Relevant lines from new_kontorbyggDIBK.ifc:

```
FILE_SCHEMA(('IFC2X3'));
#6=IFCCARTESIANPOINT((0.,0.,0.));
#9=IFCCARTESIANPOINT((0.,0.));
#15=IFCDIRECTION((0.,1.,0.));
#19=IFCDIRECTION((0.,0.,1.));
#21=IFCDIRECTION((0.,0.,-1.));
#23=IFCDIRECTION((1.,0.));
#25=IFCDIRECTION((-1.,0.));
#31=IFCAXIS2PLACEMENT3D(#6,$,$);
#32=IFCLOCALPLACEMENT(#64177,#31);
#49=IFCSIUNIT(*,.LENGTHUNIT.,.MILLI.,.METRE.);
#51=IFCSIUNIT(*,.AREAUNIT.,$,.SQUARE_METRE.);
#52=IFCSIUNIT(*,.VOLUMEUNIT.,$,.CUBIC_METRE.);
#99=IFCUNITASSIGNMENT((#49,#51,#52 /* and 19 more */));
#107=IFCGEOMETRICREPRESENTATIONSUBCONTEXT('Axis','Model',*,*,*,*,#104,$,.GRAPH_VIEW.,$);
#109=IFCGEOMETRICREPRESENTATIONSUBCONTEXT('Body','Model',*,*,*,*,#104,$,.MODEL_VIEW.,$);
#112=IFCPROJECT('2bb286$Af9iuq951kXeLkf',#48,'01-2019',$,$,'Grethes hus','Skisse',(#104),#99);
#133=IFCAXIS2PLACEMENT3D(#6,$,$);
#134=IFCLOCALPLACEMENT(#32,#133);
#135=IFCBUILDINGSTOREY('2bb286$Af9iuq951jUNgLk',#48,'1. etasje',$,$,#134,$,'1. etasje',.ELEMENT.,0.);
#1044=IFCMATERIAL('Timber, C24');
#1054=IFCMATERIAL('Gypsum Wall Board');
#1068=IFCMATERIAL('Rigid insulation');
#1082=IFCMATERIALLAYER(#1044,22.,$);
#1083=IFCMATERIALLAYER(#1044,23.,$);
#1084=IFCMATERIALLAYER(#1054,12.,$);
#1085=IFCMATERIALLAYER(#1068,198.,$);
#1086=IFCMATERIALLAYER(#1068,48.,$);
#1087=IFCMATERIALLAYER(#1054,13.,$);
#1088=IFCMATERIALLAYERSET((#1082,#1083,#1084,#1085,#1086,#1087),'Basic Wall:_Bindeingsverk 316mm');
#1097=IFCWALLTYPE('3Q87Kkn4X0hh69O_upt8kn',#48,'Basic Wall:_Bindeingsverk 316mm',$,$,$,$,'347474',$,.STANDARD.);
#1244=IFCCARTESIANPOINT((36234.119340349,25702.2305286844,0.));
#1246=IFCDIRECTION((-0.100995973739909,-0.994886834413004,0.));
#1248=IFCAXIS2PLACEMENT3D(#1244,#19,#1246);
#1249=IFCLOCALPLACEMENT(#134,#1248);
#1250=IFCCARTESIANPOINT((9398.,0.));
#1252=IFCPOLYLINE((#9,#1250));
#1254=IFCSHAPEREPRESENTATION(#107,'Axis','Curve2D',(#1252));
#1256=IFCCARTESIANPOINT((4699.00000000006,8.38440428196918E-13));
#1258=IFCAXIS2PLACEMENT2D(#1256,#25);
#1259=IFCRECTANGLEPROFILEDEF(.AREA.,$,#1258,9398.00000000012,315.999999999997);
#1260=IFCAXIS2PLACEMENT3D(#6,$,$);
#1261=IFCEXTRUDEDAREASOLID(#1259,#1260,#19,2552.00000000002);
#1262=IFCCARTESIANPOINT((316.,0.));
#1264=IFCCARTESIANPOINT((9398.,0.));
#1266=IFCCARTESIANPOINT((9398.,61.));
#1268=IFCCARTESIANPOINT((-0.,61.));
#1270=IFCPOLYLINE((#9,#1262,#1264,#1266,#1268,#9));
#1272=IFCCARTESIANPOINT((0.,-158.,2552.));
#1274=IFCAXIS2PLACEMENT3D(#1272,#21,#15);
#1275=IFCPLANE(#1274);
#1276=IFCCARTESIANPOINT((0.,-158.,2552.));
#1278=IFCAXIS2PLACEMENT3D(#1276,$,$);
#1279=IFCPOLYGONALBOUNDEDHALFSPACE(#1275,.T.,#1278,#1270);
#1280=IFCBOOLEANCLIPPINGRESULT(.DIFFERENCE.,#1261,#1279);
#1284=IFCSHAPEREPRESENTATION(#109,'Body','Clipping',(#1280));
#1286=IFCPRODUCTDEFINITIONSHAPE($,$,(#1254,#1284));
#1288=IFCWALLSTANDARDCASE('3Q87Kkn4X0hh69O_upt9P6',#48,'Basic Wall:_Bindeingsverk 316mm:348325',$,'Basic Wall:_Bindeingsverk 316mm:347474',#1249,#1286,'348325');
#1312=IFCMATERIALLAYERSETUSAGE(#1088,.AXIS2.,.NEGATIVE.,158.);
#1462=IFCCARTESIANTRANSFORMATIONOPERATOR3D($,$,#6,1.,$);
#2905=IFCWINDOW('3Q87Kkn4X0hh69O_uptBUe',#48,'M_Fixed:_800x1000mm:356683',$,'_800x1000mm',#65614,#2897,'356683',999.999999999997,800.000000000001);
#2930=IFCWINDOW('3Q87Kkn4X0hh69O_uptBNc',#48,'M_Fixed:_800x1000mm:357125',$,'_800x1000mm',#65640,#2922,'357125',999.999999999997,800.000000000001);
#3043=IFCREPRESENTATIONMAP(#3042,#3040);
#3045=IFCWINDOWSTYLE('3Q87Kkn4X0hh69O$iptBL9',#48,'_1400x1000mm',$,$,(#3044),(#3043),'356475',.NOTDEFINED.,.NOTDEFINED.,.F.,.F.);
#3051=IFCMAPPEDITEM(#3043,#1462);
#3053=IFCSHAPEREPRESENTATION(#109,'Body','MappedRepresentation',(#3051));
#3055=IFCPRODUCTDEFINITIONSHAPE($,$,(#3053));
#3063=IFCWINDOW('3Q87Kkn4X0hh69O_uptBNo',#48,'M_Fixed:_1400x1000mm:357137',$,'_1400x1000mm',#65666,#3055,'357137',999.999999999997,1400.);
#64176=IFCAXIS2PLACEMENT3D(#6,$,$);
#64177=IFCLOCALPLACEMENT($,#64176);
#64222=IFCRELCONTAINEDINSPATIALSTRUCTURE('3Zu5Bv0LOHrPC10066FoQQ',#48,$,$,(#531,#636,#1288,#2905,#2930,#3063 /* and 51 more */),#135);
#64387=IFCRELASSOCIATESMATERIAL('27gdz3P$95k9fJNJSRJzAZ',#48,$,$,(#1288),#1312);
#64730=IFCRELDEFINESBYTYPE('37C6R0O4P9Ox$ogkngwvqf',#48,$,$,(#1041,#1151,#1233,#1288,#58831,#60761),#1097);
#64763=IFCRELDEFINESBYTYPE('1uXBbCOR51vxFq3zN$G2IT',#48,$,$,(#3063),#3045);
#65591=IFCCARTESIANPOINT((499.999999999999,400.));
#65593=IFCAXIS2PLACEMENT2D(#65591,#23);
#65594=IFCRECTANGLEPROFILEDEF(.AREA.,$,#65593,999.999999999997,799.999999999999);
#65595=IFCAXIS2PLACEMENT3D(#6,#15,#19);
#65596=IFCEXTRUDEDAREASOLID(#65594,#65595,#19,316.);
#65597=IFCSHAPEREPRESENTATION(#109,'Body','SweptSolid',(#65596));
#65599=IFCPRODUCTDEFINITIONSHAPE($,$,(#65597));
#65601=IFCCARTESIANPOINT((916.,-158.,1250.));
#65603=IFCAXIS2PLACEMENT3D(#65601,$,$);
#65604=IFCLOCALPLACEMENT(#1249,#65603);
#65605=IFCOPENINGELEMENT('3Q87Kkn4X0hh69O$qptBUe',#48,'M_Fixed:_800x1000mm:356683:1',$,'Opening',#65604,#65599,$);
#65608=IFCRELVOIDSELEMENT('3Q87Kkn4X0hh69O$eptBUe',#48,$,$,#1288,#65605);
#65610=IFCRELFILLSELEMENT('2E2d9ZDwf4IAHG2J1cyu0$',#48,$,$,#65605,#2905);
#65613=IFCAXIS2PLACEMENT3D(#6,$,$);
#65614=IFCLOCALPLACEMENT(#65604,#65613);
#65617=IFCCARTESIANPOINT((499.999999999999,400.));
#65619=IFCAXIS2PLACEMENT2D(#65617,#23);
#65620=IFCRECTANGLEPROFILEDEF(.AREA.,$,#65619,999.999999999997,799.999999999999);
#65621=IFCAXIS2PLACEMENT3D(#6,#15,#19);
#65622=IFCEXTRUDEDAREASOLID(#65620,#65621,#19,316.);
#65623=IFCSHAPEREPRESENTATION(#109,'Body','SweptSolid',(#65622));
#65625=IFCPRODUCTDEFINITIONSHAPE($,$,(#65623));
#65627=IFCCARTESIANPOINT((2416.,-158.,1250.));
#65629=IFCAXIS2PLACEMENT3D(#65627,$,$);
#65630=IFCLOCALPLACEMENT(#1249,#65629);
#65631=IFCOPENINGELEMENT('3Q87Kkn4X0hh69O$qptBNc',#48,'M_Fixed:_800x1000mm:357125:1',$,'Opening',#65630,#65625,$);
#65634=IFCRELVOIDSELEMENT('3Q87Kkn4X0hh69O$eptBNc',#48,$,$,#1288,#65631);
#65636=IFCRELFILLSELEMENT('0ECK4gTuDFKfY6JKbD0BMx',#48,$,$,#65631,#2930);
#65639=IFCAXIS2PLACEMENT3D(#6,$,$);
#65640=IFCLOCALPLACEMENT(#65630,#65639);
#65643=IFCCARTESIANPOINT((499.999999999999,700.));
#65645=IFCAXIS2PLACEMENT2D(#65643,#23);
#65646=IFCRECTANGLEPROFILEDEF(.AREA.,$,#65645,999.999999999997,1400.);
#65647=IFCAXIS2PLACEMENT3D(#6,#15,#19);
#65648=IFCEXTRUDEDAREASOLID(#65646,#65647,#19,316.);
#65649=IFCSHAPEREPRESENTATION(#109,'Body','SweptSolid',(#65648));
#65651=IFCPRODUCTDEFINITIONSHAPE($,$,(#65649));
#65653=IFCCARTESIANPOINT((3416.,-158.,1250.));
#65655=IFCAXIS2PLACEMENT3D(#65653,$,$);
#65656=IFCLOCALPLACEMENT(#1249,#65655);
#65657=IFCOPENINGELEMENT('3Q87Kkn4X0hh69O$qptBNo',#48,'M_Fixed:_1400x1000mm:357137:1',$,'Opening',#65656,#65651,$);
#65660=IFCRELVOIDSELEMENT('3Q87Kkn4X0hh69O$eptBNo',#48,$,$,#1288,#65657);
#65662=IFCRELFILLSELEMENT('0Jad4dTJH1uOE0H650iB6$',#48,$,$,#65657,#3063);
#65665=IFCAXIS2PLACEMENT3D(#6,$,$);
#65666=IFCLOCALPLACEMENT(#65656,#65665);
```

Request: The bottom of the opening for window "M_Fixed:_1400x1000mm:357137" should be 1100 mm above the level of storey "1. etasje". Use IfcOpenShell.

```python
import numpy as np
import ifcopenshell
import ifcopenshell.api.geometry
import ifcopenshell.geom
import ifcopenshell.util.element
import ifcopenshell.util.placement
import ifcopenshell.util.shape
import ifcopenshell.util.unit

model = ifcopenshell.open("new_kontorbyggDIBK.ifc")
unit_scale = ifcopenshell.util.unit.calculate_unit_scale(model)

window = model.by_guid("3Q87Kkn4X0hh69O_uptBNo")
opening = window.FillsVoids[0].RelatingOpeningElement
storey = ifcopenshell.util.element.get_container(window, ifc_class="IfcBuildingStorey")
level = ifcopenshell.util.placement.get_local_placement(storey.ObjectPlacement)[2, 3]

# The opening's origin need not be at the sill, so measure its lowest point.
shape = ifcopenshell.geom.create_shape(ifcopenshell.geom.settings(), opening)
bottom = ifcopenshell.util.shape.get_shape_bottom_elevation(shape, shape.geometry) / unit_scale
dz = level + 1.1 / unit_scale - bottom

shift = np.array([0.0, 0.0, dz])
# The window is placed relative to its opening, so it follows when the opening moves.
matrix = ifcopenshell.util.placement.get_local_placement(opening.ObjectPlacement)
matrix[:3, 3] += shift
ifcopenshell.api.geometry.edit_object_placement(
    model, product=opening, matrix=matrix, is_si=False, should_transform_children=True
)

print(f"moved by {dz * unit_scale:+.3f} m")

model.write("new_kontorbyggDIBK-out.ifc")
```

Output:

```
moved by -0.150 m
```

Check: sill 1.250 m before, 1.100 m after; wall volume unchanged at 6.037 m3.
